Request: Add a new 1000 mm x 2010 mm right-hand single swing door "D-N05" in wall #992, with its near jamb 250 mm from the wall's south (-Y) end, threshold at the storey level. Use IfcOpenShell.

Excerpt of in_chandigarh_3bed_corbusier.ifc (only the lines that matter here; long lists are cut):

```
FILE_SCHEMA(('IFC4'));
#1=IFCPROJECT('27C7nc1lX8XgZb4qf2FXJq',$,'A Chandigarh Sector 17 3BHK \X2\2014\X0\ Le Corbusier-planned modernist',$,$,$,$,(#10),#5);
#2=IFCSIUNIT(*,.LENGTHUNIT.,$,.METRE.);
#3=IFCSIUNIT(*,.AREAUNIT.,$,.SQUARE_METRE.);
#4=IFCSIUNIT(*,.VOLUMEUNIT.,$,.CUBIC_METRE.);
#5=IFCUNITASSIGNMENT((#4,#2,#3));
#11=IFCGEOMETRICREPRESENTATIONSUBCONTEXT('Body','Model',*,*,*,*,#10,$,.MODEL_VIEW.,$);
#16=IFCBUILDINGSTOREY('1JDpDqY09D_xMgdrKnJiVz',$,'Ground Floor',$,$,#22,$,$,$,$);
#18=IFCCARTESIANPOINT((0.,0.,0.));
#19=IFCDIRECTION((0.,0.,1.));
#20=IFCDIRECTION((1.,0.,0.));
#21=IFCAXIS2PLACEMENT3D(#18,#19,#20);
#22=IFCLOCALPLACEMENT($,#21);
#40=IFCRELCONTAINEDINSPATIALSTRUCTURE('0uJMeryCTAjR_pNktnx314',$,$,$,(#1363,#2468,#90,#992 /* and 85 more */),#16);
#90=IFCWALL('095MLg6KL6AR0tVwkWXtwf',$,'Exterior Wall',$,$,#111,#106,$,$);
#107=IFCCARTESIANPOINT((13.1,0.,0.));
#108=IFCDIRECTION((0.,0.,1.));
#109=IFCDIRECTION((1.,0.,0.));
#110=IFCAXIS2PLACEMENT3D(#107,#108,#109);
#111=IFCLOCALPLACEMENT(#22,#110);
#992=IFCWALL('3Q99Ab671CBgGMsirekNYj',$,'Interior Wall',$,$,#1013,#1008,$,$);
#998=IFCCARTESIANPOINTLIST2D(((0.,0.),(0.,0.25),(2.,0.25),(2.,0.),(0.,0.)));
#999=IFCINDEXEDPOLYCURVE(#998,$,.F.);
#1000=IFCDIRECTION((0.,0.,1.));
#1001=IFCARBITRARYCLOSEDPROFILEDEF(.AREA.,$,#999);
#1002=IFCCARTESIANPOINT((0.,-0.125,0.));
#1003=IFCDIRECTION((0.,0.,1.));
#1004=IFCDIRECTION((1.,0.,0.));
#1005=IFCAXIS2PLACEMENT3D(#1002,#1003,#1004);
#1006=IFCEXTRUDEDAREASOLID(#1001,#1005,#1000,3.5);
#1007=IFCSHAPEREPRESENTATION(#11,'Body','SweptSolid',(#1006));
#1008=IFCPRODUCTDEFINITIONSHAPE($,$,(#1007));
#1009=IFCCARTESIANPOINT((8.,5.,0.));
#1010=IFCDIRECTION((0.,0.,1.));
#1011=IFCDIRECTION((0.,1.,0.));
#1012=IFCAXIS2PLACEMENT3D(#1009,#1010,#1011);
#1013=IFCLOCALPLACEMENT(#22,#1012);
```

```python
import numpy as np
import ifcopenshell
import ifcopenshell.api.feature
import ifcopenshell.api.geometry
import ifcopenshell.api.root
import ifcopenshell.api.spatial
import ifcopenshell.geom
import ifcopenshell.util.element
import ifcopenshell.util.placement
import ifcopenshell.util.representation
import ifcopenshell.util.shape
import ifcopenshell.util.unit

model = ifcopenshell.open("in_chandigarh_3bed_corbusier.ifc")
unit_scale = ifcopenshell.util.unit.calculate_unit_scale(model)
settings = ifcopenshell.geom.settings()


def volume(element):
    """Net volume in cubic metres, openings subtracted."""
    shape = ifcopenshell.geom.create_shape(settings, element)
    return ifcopenshell.util.shape.get_volume(shape.geometry)


wall = model.by_guid("3Q99Ab671CBgGMsirekNYj")
storey = ifcopenshell.util.element.get_container(wall, ifc_class="IfcBuildingStorey")
context = ifcopenshell.util.representation.get_context(model, "Model", "Body", "MODEL_VIEW")
before = volume(wall)

width, height, from_end, sill = 1, 2.01, 0.25, 0.0  # metres

# The wall runs along its own X axis, and the end named is its -X end.
wall_shape = ifcopenshell.geom.create_shape(settings, wall)
x, y, z = ifcopenshell.util.shape.get_vertices(wall_shape.geometry).T
start = x.min() + from_end
face, thickness = float(y.min()), float(y.max() - y.min())
wall_matrix = ifcopenshell.util.placement.get_local_placement(wall.ObjectPlacement)
level = ifcopenshell.util.placement.get_local_placement(storey.ObjectPlacement)[2, 3]


def in_wall(x, y):
    """Placement at x, y metres in the wall's axes, at sill height."""
    matrix = wall_matrix.copy()
    matrix[:, 3] = wall_matrix @ np.array([x / unit_scale, y / unit_scale, 0.0, 1.0])
    matrix[2, 3] = level + sill / unit_scale
    return matrix


# Opening: a box that overshoots both wall faces by 50 mm.
opening = ifcopenshell.api.root.create_entity(model, ifc_class="IfcOpeningElement", predefined_type="OPENING")
box = ifcopenshell.api.geometry.add_wall_representation(
    model, context=context, length=width, height=height, thickness=thickness + 0.1
)
ifcopenshell.api.geometry.assign_representation(model, product=opening, representation=box)
ifcopenshell.api.geometry.edit_object_placement(model, product=opening, matrix=in_wall(start, face - 0.05), is_si=False)
ifcopenshell.api.feature.add_feature(model, feature=opening, element=wall)

door = ifcopenshell.api.root.create_entity(model, ifc_class="IfcDoor", name="D-N05", predefined_type="DOOR")
door.OverallWidth, door.OverallHeight = width / unit_scale, height / unit_scale
door.OperationType = "SINGLE_SWING_RIGHT"
body = ifcopenshell.api.geometry.add_door_representation(
    model,
    context=context,
    overall_width=door.OverallWidth,
    overall_height=door.OverallHeight,
    operation_type="SINGLE_SWING_RIGHT",
    lining_properties={"LiningDepth": thickness / unit_scale, "ThresholdDepth": thickness / unit_scale},
)
ifcopenshell.api.geometry.assign_representation(model, product=door, representation=body)
ifcopenshell.api.spatial.assign_container(model, products=[door], relating_structure=storey)
ifcopenshell.api.feature.add_filling(model, opening=opening, element=door)

# The lining spans the wall, so the door starts at the wall face.
ifcopenshell.api.geometry.edit_object_placement(model, product=door, matrix=in_wall(start, face), is_si=False)

after = volume(wall)

print(f"wall volume {before:.3f} -> {after:.3f} m3")

model.write("in_chandigarh_3bed_corbusier_updated.ifc")
```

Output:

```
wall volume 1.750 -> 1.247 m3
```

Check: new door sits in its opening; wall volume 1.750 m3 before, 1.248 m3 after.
